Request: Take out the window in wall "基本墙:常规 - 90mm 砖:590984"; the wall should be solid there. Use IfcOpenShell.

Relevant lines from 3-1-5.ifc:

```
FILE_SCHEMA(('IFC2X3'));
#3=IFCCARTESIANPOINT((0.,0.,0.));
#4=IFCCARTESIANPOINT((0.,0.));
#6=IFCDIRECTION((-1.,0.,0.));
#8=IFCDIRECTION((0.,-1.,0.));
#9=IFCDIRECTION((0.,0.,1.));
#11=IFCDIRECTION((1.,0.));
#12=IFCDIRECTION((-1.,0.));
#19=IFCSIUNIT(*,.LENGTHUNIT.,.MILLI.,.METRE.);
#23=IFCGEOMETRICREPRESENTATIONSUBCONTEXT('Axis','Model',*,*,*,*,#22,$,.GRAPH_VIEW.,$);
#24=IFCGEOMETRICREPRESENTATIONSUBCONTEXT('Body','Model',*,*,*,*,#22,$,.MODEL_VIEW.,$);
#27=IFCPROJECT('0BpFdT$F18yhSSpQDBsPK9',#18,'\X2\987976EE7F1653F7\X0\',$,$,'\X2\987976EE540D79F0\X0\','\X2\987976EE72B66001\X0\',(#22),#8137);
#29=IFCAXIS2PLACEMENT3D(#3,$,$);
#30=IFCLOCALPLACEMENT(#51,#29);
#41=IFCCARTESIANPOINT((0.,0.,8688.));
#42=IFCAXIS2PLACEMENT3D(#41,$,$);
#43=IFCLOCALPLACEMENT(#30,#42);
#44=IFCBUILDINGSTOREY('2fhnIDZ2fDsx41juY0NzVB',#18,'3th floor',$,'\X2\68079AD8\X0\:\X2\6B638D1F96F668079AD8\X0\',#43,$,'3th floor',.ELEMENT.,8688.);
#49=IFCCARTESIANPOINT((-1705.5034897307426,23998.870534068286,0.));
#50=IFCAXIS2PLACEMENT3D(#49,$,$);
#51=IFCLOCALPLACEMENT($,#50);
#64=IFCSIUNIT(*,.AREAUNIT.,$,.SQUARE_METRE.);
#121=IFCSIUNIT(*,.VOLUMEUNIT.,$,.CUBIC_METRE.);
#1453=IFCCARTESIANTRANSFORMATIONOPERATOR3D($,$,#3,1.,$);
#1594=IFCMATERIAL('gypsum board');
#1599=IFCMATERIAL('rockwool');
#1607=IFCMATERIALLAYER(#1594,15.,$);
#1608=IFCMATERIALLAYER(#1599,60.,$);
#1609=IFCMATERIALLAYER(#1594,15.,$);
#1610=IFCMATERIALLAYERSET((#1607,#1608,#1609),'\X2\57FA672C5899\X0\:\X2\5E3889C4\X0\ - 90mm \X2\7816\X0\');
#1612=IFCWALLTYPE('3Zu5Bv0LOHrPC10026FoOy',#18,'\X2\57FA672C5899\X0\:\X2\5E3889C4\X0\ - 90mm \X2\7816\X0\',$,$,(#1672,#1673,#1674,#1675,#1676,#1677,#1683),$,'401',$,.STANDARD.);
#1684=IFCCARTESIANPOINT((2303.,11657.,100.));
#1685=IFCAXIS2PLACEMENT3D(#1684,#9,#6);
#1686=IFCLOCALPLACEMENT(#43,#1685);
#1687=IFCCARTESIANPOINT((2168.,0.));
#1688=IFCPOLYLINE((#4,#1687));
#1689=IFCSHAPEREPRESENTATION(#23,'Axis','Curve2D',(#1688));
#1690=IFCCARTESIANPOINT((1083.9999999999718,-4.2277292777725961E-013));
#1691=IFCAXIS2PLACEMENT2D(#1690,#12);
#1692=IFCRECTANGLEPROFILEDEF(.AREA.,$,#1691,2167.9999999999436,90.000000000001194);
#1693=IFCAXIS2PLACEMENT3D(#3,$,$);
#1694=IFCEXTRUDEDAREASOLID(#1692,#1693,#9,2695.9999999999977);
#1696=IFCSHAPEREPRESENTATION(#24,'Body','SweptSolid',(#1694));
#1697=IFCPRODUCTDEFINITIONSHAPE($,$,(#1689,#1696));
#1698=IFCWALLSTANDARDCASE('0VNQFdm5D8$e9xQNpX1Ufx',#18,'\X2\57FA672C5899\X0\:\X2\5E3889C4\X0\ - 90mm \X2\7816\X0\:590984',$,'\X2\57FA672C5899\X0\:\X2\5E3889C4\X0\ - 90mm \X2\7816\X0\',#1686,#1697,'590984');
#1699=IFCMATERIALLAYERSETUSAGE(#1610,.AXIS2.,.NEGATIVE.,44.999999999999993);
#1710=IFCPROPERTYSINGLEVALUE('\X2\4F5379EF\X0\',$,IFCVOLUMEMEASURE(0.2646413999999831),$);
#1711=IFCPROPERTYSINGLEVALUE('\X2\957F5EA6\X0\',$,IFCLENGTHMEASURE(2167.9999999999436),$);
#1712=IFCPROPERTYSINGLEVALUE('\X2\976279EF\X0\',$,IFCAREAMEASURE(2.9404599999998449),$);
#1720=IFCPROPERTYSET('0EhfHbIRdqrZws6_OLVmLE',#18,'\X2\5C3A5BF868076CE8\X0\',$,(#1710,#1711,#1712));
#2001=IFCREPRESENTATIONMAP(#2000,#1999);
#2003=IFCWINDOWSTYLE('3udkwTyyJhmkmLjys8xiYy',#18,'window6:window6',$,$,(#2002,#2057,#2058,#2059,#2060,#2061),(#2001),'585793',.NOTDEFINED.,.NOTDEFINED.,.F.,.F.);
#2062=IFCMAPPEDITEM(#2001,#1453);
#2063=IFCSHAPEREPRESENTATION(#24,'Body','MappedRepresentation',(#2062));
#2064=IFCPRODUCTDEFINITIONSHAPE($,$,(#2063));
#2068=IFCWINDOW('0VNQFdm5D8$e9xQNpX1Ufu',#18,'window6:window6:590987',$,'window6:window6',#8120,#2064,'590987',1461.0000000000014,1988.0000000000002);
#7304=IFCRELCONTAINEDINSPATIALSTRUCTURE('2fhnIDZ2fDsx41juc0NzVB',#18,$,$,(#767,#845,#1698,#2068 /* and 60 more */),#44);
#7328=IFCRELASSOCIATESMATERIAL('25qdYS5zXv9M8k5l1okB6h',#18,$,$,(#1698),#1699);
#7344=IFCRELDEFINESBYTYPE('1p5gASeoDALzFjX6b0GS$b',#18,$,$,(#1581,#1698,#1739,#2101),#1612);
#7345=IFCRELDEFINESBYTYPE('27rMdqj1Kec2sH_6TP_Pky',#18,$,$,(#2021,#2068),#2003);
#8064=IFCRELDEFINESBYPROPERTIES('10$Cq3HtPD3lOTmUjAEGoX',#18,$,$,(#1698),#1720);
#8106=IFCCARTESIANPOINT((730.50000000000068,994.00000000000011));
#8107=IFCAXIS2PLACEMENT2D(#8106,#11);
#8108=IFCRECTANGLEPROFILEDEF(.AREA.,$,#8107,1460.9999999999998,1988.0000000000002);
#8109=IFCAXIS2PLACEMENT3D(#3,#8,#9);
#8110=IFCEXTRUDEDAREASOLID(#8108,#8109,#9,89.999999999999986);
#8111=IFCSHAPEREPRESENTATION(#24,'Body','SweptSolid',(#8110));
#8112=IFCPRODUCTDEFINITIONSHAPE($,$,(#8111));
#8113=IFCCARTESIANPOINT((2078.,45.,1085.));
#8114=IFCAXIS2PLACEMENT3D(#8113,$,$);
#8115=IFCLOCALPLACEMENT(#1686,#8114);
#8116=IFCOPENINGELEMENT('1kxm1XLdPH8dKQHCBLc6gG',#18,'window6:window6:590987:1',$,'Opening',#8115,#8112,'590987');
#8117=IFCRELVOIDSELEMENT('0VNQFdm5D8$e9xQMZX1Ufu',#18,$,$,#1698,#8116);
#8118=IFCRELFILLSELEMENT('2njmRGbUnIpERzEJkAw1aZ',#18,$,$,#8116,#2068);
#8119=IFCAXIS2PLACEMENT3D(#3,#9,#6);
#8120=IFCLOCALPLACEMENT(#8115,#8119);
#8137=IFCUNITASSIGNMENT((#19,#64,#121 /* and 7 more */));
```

```python
import ifcopenshell
import ifcopenshell.api.feature
import ifcopenshell.api.pset
import ifcopenshell.api.root
import ifcopenshell.geom
import ifcopenshell.util.element
import ifcopenshell.util.shape
import ifcopenshell.util.unit

model = ifcopenshell.open("3-1-5.ifc")
area_scale = ifcopenshell.util.unit.calculate_unit_scale(model, "AREAUNIT")
volume_scale = ifcopenshell.util.unit.calculate_unit_scale(model, "VOLUMEUNIT")
settings = ifcopenshell.geom.settings()


def volume(element):
    """Net volume in cubic metres, openings subtracted."""
    shape = ifcopenshell.geom.create_shape(settings, element)
    return ifcopenshell.util.shape.get_volume(shape.geometry)


window = model.by_id(2068)
opening = window.FillsVoids[0].RelatingOpeningElement
wall = opening.VoidsElements[0].RelatingBuildingElement
before = volume(wall)

ifcopenshell.api.root.remove_product(model, product=window)
ifcopenshell.api.feature.remove_feature(model, feature=opening)

after = volume(wall)
thickness = 0.09  # wall thickness in metres

# Update the wall's stored quantities.
pset = model.by_id(ifcopenshell.util.element.get_pset(wall, "尺寸标注", should_inherit=False)["id"])
ifcopenshell.api.pset.edit_pset(model, pset=pset, properties={
    "体积": model.create_entity("IfcVolumeMeasure", after / volume_scale),
    "面积": model.create_entity("IfcAreaMeasure", after / thickness / area_scale),
})

print(f"wall volume {before:.3f} -> {after:.3f} m3")

model.write("3-1-5_edited.ifc")
```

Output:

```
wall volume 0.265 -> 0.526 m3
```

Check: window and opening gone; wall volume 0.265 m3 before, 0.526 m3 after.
